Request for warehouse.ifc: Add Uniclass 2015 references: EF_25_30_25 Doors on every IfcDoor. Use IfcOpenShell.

First a look at what the model holds.

```python
import ifcopenshell

model = ifcopenshell.open("warehouse.ifc")
print(model.schema)
print("classifications:", [c.Name for c in model.by_type("IfcClassification")])
for ifc_class in ("IfcDoor", "IfcRoof", "IfcStair", "IfcWall", "IfcWindow"):
    print(ifc_class, len(model.by_type(ifc_class)))
```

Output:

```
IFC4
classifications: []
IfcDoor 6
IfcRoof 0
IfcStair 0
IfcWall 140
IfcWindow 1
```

```python
import ifcopenshell
import ifcopenshell.api.classification

model = ifcopenshell.open("warehouse.ifc")

system = ifcopenshell.api.classification.add_classification(model, classification="Uniclass 2015")

codes = {
    "IfcDoor": ("EF_25_30_25", "Doors"),
}
for ifc_class, (code, name) in codes.items():
    products = model.by_type(ifc_class)
    ifcopenshell.api.classification.add_reference(
        model, products=products, classification=system, identification=code, name=name
    )
    print(code, len(products))

model.write("warehouse_rev.ifc")
```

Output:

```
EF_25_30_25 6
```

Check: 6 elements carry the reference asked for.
